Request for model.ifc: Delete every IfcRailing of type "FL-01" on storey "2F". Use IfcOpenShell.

First a look at what the model holds.

```python
import ifcopenshell
import ifcopenshell.util.element

model = ifcopenshell.open("model.ifc")
print(model.schema)
storey = next(s for s in model.by_type("IfcBuildingStorey") if s.Name == "2F")
railings = [e for e in ifcopenshell.util.element.get_decomposition(storey) if e.is_a("IfcRailing")]
seen = {}
for e in railings:
    element_type = ifcopenshell.util.element.get_type(e)
    name = element_type.Name if element_type not in (None, e) else None
    seen[name] = seen.get(name, 0) + 1
for name, count in sorted(seen.items(), key=str):
    print(count, "x", name)
```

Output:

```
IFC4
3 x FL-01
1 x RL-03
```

```python
import ifcopenshell
import ifcopenshell.api.root
import ifcopenshell.util.element

model = ifcopenshell.open("model.ifc")

storey = next(s for s in model.by_type("IfcBuildingStorey") if s.Name == "2F")
railings = [e for e in ifcopenshell.util.element.get_decomposition(storey) if e.is_a("IfcRailing")]
targets = [e for e in railings if (t := ifcopenshell.util.element.get_type(e)) not in (None, e) and t.Name == "FL-01"]

for e in targets:
    ifcopenshell.api.root.remove_product(model, product=e)
print(len(targets), "removed")

model.write("model_v2.ifc")
```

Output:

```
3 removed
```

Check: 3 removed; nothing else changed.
